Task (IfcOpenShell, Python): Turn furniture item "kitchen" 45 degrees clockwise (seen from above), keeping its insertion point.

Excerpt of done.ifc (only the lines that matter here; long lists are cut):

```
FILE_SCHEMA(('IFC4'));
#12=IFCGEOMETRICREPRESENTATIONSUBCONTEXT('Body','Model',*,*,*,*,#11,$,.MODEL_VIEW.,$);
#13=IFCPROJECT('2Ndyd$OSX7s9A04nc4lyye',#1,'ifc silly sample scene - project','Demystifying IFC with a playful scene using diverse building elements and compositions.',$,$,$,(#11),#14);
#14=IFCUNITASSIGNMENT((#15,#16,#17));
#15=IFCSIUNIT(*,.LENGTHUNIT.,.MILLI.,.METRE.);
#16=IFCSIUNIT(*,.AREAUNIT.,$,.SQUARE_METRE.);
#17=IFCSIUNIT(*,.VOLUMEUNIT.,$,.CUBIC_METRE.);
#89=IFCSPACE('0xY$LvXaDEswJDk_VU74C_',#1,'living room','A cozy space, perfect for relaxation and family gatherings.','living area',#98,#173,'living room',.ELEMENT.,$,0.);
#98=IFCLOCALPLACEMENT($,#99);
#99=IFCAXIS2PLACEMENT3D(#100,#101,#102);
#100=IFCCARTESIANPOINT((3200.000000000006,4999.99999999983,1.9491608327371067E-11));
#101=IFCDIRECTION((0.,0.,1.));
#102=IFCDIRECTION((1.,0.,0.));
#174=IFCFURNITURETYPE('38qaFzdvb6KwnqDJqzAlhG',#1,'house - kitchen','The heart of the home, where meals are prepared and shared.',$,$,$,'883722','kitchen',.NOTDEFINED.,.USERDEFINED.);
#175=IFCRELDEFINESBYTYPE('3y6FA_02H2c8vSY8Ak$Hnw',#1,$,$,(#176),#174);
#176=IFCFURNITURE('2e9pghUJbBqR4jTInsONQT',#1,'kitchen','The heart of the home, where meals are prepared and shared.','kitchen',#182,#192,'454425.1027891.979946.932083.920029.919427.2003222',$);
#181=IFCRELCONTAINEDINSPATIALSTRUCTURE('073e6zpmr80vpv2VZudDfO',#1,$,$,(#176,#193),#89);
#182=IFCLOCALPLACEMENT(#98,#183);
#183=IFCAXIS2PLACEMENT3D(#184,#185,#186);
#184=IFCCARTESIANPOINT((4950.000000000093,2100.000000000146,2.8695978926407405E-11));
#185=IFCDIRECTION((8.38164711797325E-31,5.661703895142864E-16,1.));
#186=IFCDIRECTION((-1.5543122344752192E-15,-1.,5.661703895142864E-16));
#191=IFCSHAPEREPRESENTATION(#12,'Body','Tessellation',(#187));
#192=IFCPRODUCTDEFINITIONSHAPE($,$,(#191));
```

```python
import ifcopenshell
import ifcopenshell.api.geometry
import ifcopenshell.util.placement

model = ifcopenshell.open("done.ifc")

item = model.by_guid("2e9pghUJbBqR4jTInsONQT")
matrix = ifcopenshell.util.placement.get_local_placement(item.ObjectPlacement)
matrix = matrix @ ifcopenshell.util.placement.rotation(-45, "Z")
ifcopenshell.api.geometry.edit_object_placement(model, product=item, matrix=matrix, is_si=False)

print(ifcopenshell.util.placement.get_local_placement(item.ObjectPlacement).round(3) + 0.0)

model.write("done_updated.ifc")
```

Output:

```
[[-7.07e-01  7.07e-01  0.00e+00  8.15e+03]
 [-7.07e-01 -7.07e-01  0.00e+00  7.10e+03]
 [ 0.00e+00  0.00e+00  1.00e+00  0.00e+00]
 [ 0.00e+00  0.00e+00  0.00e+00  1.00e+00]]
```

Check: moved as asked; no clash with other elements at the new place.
